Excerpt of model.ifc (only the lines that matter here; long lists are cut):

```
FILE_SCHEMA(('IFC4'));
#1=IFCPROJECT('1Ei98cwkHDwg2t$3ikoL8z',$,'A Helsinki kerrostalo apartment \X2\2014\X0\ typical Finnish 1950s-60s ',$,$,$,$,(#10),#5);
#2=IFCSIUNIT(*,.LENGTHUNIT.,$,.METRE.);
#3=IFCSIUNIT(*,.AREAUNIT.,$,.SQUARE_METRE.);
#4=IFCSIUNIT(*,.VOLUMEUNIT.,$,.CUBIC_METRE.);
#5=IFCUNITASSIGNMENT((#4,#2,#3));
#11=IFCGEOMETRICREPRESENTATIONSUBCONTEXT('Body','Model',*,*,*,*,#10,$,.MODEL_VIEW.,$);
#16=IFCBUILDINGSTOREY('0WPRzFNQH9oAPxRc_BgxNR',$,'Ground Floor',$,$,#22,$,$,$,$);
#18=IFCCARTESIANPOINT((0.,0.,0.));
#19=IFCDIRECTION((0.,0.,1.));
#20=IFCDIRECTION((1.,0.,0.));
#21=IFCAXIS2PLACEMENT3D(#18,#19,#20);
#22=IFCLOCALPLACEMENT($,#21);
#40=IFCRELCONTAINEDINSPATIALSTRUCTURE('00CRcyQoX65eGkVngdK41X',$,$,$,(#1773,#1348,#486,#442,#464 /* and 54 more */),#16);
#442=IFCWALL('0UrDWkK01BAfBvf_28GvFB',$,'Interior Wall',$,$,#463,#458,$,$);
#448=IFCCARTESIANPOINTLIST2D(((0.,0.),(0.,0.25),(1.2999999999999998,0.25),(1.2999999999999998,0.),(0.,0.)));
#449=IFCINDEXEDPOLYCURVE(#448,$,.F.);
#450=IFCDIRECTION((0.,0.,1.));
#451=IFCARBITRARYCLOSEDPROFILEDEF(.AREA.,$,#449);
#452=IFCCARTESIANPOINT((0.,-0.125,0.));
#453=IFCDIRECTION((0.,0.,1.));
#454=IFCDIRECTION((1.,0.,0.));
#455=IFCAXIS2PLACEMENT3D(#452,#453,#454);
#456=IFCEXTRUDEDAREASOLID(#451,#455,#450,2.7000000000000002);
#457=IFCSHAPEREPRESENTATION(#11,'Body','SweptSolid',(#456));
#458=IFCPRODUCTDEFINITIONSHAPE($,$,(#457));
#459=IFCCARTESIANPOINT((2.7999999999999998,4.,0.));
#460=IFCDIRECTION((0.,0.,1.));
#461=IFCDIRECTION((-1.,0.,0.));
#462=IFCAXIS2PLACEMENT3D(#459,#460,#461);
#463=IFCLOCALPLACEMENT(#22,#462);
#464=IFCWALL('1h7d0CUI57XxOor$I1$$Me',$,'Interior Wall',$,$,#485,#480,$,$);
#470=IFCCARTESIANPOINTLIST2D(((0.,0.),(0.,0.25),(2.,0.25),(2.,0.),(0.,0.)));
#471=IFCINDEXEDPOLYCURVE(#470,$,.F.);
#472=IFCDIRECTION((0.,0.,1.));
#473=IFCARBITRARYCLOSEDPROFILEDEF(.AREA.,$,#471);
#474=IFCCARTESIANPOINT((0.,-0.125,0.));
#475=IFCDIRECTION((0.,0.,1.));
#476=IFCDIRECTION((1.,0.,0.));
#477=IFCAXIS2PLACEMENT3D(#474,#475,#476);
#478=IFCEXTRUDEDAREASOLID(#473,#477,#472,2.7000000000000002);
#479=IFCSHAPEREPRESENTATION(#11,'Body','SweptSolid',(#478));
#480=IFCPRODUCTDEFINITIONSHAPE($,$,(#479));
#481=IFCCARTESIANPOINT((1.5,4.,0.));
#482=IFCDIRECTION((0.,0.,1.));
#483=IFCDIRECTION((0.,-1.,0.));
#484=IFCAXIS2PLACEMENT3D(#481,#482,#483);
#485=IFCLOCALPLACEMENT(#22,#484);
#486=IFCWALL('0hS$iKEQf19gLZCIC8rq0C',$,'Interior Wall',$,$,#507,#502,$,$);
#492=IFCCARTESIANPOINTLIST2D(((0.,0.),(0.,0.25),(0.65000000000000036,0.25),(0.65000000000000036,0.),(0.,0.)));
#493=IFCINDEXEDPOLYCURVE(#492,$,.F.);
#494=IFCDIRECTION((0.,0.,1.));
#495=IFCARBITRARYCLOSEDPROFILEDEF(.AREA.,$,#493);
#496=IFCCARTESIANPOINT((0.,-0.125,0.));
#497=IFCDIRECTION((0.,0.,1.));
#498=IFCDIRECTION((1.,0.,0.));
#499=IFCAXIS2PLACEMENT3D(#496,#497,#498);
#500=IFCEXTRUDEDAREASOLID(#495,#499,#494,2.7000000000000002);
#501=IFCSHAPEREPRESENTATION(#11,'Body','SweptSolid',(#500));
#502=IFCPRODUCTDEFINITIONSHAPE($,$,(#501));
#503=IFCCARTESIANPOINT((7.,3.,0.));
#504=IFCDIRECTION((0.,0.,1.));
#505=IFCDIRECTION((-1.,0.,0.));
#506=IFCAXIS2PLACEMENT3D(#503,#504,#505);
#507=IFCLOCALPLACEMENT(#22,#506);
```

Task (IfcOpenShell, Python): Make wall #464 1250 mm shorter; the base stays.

```python
import ifcopenshell
import ifcopenshell.geom
import ifcopenshell.util.representation
import ifcopenshell.util.shape

model = ifcopenshell.open("model.ifc")
settings = ifcopenshell.geom.settings()


def volume(element):
    """Net volume in cubic metres, openings subtracted."""
    shape = ifcopenshell.geom.create_shape(settings, element)
    return ifcopenshell.util.shape.get_volume(shape.geometry)


wall = model.by_guid("1h7d0CUI57XxOor$I1$$Me")
before = volume(wall)

body = ifcopenshell.util.representation.get_representation(wall, "Model", "Body")
solid = body.Items[0]
old_height = solid.Depth
solid.Depth -= 1.25
after = volume(wall)

print(f"height {old_height:g} -> {solid.Depth:g}, volume {before:.3f} -> {after:.3f} m3")

model.write("model_edited.ifc")
```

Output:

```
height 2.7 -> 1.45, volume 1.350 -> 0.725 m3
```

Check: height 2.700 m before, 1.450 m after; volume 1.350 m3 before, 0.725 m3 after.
